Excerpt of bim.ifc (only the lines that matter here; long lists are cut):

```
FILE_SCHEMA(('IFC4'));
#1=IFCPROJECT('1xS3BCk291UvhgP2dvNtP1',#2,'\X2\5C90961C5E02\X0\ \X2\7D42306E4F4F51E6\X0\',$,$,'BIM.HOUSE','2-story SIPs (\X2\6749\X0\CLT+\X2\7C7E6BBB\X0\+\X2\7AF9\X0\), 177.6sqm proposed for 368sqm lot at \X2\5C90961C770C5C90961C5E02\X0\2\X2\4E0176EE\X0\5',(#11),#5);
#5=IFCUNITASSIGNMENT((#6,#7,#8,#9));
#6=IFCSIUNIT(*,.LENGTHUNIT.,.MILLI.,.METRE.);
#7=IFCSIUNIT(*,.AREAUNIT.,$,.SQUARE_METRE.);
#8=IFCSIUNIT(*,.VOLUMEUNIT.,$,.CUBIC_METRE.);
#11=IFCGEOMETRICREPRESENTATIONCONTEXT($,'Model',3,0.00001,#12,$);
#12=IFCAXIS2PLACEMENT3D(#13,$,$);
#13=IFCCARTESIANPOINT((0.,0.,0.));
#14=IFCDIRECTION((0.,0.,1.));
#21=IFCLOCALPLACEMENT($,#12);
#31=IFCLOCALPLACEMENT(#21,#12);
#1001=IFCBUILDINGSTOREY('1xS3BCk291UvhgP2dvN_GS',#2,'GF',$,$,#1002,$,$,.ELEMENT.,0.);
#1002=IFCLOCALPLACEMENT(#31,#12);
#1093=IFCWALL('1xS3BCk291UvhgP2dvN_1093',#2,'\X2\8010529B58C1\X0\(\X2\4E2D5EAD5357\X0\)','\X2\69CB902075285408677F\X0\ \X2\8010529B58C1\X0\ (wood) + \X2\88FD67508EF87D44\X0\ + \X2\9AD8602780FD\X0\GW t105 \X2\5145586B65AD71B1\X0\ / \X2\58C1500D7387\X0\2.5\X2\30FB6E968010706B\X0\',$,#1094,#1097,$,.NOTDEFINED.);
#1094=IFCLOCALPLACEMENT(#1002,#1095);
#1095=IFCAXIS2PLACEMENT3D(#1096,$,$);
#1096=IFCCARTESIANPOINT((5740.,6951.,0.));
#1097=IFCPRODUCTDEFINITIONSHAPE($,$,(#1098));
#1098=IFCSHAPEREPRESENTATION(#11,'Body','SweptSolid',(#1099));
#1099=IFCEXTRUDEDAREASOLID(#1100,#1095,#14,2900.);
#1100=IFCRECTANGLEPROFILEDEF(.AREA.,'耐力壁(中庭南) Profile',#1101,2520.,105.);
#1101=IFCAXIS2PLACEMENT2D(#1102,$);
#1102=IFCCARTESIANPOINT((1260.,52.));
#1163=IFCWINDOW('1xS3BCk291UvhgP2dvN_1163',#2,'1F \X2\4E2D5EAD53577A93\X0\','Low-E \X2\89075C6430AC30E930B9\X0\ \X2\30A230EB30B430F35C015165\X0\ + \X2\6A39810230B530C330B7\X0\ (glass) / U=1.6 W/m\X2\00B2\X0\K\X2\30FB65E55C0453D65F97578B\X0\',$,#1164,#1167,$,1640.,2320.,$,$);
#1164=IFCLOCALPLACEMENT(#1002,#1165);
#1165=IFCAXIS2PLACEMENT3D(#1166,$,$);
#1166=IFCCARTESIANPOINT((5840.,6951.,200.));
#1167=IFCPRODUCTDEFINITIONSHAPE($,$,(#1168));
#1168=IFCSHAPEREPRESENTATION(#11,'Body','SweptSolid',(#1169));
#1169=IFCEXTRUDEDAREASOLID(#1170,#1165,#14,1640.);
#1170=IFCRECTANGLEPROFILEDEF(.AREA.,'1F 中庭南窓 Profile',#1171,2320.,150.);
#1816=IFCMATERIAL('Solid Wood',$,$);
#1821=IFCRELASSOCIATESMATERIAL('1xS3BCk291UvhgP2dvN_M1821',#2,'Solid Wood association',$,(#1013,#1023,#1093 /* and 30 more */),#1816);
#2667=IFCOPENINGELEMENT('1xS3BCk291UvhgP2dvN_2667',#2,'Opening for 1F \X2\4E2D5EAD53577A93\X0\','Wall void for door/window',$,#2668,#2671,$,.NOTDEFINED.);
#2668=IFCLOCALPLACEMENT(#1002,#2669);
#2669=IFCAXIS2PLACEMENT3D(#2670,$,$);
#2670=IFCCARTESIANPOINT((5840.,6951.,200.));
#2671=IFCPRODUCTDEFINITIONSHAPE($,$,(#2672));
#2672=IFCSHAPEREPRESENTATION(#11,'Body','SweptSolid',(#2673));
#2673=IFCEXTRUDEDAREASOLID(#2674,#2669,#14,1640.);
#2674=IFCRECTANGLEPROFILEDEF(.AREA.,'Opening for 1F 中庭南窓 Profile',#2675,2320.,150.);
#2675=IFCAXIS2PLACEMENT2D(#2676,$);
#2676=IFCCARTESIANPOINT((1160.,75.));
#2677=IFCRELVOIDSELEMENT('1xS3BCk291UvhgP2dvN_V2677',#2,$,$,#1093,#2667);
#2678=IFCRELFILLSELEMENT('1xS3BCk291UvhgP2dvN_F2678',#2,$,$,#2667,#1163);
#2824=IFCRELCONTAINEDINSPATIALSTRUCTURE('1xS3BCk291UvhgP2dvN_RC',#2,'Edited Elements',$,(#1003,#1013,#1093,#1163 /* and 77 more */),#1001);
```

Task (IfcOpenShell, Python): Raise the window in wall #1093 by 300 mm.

```python
import numpy as np
import ifcopenshell
import ifcopenshell.api.geometry
import ifcopenshell.util.placement
import ifcopenshell.util.unit

model = ifcopenshell.open("bim.ifc")
unit_scale = ifcopenshell.util.unit.calculate_unit_scale(model)

window = model.by_id(1163)
opening = window.FillsVoids[0].RelatingOpeningElement
dz = 0.3 / unit_scale

shift = np.array([0.0, 0.0, dz])
# The window is not placed relative to its opening, so move both.
for product in (opening, window):
    matrix = ifcopenshell.util.placement.get_local_placement(product.ObjectPlacement)
    matrix[:3, 3] += shift
    ifcopenshell.api.geometry.edit_object_placement(model, product=product, matrix=matrix, is_si=False)

print(f"moved by {dz * unit_scale:+.3f} m")

model.write("bim_updated.ifc")
```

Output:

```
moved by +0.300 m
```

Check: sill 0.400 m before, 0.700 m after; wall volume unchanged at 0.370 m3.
